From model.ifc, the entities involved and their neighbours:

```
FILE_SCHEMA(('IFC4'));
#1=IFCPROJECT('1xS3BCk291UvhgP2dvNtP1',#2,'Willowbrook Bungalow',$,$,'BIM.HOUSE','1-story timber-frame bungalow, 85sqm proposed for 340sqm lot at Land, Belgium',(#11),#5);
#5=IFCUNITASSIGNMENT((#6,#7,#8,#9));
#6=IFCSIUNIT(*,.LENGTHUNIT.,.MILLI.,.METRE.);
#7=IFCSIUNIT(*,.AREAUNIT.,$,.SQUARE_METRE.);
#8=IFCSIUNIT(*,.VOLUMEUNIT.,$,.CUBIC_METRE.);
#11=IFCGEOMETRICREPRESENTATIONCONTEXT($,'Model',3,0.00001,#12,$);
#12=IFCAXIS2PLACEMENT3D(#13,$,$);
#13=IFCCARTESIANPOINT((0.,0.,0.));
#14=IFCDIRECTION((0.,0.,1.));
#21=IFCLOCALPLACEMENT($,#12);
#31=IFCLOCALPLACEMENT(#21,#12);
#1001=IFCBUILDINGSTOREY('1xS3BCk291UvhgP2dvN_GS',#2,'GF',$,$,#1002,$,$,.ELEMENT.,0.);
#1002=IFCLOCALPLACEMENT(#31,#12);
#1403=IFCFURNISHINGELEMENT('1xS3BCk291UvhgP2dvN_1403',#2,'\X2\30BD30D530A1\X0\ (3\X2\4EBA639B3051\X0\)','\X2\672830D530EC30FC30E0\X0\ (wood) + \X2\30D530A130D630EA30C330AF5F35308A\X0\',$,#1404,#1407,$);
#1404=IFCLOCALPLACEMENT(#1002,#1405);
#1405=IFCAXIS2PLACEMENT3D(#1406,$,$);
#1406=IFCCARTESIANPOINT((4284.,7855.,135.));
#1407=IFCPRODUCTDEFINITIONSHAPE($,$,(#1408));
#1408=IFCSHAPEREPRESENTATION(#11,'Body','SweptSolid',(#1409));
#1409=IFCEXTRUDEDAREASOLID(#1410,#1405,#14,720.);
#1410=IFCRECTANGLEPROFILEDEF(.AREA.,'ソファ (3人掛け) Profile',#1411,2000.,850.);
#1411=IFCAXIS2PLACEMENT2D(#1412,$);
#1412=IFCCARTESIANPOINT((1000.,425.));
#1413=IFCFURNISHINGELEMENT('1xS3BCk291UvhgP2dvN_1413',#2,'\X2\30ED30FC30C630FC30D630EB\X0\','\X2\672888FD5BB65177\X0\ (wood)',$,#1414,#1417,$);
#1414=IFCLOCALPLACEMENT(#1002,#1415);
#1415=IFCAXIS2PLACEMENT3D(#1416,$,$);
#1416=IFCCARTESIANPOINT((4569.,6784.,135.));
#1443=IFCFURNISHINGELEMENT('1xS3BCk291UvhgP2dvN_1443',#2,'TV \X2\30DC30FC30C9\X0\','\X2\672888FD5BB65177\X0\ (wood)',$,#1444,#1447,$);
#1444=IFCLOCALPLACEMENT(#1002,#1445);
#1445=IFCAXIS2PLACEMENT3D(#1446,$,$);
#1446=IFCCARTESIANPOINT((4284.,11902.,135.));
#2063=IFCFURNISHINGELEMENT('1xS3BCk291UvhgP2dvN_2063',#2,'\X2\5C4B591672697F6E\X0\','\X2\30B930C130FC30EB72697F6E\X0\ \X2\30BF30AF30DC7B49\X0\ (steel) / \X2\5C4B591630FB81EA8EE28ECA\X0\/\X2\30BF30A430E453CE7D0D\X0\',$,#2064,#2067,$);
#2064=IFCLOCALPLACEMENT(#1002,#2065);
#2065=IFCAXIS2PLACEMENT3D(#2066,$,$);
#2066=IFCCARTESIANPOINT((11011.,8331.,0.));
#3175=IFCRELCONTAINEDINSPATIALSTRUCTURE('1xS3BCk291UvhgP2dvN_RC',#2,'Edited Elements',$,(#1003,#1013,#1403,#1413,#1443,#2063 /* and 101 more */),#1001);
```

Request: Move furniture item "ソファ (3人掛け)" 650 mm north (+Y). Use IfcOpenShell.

```python
import ifcopenshell
import ifcopenshell.api.geometry
import ifcopenshell.util.placement

model = ifcopenshell.open("model.ifc")

item = model.by_guid("1xS3BCk291UvhgP2dvN_1403")
matrix = ifcopenshell.util.placement.get_local_placement(item.ObjectPlacement)
matrix[1, 3] += 650.0
ifcopenshell.api.geometry.edit_object_placement(model, product=item, matrix=matrix, is_si=False)

print(ifcopenshell.util.placement.get_local_placement(item.ObjectPlacement).round(3) + 0.0)

model.write("model_updated.ifc")
```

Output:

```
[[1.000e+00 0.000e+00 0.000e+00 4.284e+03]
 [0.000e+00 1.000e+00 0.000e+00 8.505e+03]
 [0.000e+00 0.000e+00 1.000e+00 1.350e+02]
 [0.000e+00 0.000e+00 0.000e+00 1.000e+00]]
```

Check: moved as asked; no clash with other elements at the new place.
